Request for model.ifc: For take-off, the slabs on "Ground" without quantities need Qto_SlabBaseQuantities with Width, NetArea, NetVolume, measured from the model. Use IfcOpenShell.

First a look at what the model holds.

```python
import ifcopenshell
import ifcopenshell.util.element
import ifcopenshell.util.unit

model = ifcopenshell.open("model.ifc")
print(model.schema)
for unit_type in ("LENGTHUNIT", "AREAUNIT", "VOLUMEUNIT"):
    print(unit_type, ifcopenshell.util.unit.calculate_unit_scale(model, unit_type))
storey = next(s for s in model.by_type("IfcBuildingStorey") if s.Name == "Ground")
slabs = [e for e in ifcopenshell.util.element.get_decomposition(storey) if e.is_a("IfcSlab")]
for e in sorted(slabs, key=lambda e: e.id()):
    print(e.id(), e.is_a(), e.Name, list(ifcopenshell.util.element.get_psets(e, qtos_only=True)), sep=" | ")
```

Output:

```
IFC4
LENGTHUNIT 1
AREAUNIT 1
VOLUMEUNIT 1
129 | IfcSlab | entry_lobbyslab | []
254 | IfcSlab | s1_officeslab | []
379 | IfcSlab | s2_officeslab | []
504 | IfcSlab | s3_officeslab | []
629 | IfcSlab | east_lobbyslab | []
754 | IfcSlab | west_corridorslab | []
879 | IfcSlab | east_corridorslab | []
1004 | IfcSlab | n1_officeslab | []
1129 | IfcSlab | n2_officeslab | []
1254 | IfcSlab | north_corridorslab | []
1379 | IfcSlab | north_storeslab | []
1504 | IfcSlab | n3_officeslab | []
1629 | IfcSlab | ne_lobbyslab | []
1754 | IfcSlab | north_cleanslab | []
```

```python
import ifcopenshell
import ifcopenshell.api.pset
import ifcopenshell.geom
import ifcopenshell.util.element
import ifcopenshell.util.shape
import ifcopenshell.util.unit

model = ifcopenshell.open("model.ifc")
unit_scale = ifcopenshell.util.unit.calculate_unit_scale(model)
area_scale = ifcopenshell.util.unit.calculate_unit_scale(model, "AREAUNIT")
volume_scale = ifcopenshell.util.unit.calculate_unit_scale(model, "VOLUMEUNIT")
settings = ifcopenshell.geom.settings()

storey = next(s for s in model.by_type("IfcBuildingStorey") if s.Name == "Ground")
slabs = [e for e in ifcopenshell.util.element.get_decomposition(storey) if e.is_a("IfcSlab")]

for e in sorted(slabs, key=lambda e: e.id()):
    if ifcopenshell.util.element.get_psets(e, qtos_only=True, should_inherit=False):
        continue
    # Geometry comes back in metres, in the element's own axes.
    shape = ifcopenshell.geom.create_shape(settings, e)
    values = {
        "Width": ifcopenshell.util.shape.get_z(shape.geometry) / unit_scale,
        "NetArea": ifcopenshell.util.shape.get_footprint_area(shape.geometry) / area_scale,
        "NetVolume": ifcopenshell.util.shape.get_volume(shape.geometry) / volume_scale,
    }
    qto = ifcopenshell.api.pset.add_qto(model, product=e, name="Qto_SlabBaseQuantities")
    ifcopenshell.api.pset.edit_qto(model, qto=qto, properties=values)
    print(e.id(), {k: round(v, 3) for k, v in values.items()})

model.write("model-out.ifc")
```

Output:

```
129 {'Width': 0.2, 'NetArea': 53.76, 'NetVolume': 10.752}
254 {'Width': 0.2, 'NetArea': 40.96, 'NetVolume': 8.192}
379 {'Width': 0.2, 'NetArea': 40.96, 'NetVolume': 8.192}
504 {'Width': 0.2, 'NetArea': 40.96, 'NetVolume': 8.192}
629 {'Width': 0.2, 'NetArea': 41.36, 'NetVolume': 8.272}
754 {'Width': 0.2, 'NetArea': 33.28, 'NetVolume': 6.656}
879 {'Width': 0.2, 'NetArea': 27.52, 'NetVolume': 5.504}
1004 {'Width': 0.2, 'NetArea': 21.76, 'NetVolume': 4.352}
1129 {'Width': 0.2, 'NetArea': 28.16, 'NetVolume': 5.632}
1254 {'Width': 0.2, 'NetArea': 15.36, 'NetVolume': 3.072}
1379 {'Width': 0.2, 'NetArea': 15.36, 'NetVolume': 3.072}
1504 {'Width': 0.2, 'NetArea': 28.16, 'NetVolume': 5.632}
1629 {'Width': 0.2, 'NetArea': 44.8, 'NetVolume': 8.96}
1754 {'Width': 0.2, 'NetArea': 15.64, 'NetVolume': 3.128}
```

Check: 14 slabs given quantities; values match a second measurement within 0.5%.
